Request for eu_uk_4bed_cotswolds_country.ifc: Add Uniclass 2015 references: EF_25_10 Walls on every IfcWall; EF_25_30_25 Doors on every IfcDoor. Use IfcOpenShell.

First a look at what the model holds.

```python
import ifcopenshell

model = ifcopenshell.open("eu_uk_4bed_cotswolds_country.ifc")
print(model.schema)
print("classifications:", [c.Name for c in model.by_type("IfcClassification")])
for ifc_class in ("IfcDoor", "IfcRoof", "IfcStair", "IfcWall", "IfcWindow"):
    print(ifc_class, len(model.by_type(ifc_class)))
```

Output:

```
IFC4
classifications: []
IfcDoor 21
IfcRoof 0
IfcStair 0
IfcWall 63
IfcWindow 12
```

```python
import ifcopenshell
import ifcopenshell.api.classification

model = ifcopenshell.open("eu_uk_4bed_cotswolds_country.ifc")

system = ifcopenshell.api.classification.add_classification(model, classification="Uniclass 2015")

codes = {
    "IfcWall": ("EF_25_10", "Walls"),
    "IfcDoor": ("EF_25_30_25", "Doors"),
}
for ifc_class, (code, name) in codes.items():
    products = model.by_type(ifc_class)
    ifcopenshell.api.classification.add_reference(
        model, products=products, classification=system, identification=code, name=name
    )
    print(code, len(products))

model.write("eu_uk_4bed_cotswolds_country_updated.ifc")
```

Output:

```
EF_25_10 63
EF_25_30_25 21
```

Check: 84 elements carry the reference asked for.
